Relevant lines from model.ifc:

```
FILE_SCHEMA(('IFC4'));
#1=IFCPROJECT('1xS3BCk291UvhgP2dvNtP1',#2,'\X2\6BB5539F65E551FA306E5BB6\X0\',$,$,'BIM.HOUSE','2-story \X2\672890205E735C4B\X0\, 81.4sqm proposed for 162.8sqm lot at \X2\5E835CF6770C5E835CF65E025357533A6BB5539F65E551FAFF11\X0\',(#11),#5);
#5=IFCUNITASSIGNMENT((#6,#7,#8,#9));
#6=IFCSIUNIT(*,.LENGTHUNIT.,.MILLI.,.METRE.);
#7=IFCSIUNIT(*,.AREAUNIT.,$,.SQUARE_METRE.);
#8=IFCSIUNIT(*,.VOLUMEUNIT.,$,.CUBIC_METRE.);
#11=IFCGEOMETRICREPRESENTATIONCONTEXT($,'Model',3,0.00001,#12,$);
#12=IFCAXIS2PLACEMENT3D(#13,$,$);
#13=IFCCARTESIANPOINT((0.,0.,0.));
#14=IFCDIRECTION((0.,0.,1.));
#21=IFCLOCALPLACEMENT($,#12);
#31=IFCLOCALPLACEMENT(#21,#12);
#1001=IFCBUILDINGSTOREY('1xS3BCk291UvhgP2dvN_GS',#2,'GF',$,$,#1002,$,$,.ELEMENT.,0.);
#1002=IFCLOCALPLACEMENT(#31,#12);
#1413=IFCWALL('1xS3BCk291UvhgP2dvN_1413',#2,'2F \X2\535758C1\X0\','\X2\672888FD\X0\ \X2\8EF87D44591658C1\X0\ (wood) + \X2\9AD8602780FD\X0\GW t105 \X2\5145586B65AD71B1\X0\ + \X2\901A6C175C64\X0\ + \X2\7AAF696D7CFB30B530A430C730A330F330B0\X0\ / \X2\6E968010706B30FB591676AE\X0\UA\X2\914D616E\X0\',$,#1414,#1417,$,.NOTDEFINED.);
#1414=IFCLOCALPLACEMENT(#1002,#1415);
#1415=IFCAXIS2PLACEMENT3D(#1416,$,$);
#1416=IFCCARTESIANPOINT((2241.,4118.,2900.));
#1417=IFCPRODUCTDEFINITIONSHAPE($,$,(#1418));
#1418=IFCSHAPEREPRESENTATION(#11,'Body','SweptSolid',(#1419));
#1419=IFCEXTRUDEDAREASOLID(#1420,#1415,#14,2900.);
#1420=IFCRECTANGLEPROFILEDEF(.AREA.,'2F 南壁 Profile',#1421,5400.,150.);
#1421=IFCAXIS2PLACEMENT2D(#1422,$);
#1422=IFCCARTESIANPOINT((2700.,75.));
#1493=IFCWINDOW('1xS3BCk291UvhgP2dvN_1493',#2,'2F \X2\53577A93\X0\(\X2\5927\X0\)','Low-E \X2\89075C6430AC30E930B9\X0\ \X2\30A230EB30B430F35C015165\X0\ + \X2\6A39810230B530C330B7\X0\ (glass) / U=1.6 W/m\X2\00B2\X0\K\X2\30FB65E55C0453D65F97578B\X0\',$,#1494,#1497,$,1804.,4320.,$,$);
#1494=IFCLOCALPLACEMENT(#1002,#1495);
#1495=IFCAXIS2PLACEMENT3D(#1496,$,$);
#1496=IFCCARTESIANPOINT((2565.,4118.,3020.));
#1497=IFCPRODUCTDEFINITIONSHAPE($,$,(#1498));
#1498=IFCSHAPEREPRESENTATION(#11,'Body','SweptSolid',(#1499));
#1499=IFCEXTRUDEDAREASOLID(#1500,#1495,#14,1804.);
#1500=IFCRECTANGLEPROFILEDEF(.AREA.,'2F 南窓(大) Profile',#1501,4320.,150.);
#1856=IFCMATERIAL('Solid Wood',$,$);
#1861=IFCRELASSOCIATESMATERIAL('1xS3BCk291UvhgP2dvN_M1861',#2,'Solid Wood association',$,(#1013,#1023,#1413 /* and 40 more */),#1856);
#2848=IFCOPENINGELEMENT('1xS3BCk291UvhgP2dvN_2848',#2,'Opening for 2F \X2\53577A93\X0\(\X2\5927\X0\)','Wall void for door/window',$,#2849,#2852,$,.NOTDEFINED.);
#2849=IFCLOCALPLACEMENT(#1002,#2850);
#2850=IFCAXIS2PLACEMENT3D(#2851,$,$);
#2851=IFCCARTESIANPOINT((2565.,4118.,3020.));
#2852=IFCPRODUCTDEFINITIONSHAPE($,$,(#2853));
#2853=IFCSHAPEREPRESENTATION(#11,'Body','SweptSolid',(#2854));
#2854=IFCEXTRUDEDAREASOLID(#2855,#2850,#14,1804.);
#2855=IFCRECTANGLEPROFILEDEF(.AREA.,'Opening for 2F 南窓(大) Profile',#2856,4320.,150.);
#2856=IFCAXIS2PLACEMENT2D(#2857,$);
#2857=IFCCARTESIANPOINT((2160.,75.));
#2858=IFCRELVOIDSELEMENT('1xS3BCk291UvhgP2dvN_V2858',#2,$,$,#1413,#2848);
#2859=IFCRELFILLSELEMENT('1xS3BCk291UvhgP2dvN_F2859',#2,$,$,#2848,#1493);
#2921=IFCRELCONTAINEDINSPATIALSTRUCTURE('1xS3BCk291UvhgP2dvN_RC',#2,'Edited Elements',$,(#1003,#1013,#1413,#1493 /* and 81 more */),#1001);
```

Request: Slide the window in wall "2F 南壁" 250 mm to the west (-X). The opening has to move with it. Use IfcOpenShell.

```python
import ifcopenshell
import ifcopenshell.api.geometry
import ifcopenshell.util.placement
import ifcopenshell.util.unit

model = ifcopenshell.open("model.ifc")
unit_scale = ifcopenshell.util.unit.calculate_unit_scale(model)

window = model.by_id(1493)
opening = window.FillsVoids[0].RelatingOpeningElement
wall = opening.VoidsElements[0].RelatingBuildingElement

wall_matrix = ifcopenshell.util.placement.get_local_placement(wall.ObjectPlacement)
shift = wall_matrix[:3, 0] * -0.25 / unit_scale
before = ifcopenshell.util.placement.get_local_placement(window.ObjectPlacement)[:3, 3].copy()

# The window is not placed relative to its opening, so move both.
for product in (opening, window):
    matrix = ifcopenshell.util.placement.get_local_placement(product.ObjectPlacement)
    matrix[:3, 3] += shift
    ifcopenshell.api.geometry.edit_object_placement(model, product=product, matrix=matrix, is_si=False)

after = ifcopenshell.util.placement.get_local_placement(window.ObjectPlacement)[:3, 3]
print("window moved by", (after - before).round(3) + 0.0)

model.write("model_updated.ifc")
```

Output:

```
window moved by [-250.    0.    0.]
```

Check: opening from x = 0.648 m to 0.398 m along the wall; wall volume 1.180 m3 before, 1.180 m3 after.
